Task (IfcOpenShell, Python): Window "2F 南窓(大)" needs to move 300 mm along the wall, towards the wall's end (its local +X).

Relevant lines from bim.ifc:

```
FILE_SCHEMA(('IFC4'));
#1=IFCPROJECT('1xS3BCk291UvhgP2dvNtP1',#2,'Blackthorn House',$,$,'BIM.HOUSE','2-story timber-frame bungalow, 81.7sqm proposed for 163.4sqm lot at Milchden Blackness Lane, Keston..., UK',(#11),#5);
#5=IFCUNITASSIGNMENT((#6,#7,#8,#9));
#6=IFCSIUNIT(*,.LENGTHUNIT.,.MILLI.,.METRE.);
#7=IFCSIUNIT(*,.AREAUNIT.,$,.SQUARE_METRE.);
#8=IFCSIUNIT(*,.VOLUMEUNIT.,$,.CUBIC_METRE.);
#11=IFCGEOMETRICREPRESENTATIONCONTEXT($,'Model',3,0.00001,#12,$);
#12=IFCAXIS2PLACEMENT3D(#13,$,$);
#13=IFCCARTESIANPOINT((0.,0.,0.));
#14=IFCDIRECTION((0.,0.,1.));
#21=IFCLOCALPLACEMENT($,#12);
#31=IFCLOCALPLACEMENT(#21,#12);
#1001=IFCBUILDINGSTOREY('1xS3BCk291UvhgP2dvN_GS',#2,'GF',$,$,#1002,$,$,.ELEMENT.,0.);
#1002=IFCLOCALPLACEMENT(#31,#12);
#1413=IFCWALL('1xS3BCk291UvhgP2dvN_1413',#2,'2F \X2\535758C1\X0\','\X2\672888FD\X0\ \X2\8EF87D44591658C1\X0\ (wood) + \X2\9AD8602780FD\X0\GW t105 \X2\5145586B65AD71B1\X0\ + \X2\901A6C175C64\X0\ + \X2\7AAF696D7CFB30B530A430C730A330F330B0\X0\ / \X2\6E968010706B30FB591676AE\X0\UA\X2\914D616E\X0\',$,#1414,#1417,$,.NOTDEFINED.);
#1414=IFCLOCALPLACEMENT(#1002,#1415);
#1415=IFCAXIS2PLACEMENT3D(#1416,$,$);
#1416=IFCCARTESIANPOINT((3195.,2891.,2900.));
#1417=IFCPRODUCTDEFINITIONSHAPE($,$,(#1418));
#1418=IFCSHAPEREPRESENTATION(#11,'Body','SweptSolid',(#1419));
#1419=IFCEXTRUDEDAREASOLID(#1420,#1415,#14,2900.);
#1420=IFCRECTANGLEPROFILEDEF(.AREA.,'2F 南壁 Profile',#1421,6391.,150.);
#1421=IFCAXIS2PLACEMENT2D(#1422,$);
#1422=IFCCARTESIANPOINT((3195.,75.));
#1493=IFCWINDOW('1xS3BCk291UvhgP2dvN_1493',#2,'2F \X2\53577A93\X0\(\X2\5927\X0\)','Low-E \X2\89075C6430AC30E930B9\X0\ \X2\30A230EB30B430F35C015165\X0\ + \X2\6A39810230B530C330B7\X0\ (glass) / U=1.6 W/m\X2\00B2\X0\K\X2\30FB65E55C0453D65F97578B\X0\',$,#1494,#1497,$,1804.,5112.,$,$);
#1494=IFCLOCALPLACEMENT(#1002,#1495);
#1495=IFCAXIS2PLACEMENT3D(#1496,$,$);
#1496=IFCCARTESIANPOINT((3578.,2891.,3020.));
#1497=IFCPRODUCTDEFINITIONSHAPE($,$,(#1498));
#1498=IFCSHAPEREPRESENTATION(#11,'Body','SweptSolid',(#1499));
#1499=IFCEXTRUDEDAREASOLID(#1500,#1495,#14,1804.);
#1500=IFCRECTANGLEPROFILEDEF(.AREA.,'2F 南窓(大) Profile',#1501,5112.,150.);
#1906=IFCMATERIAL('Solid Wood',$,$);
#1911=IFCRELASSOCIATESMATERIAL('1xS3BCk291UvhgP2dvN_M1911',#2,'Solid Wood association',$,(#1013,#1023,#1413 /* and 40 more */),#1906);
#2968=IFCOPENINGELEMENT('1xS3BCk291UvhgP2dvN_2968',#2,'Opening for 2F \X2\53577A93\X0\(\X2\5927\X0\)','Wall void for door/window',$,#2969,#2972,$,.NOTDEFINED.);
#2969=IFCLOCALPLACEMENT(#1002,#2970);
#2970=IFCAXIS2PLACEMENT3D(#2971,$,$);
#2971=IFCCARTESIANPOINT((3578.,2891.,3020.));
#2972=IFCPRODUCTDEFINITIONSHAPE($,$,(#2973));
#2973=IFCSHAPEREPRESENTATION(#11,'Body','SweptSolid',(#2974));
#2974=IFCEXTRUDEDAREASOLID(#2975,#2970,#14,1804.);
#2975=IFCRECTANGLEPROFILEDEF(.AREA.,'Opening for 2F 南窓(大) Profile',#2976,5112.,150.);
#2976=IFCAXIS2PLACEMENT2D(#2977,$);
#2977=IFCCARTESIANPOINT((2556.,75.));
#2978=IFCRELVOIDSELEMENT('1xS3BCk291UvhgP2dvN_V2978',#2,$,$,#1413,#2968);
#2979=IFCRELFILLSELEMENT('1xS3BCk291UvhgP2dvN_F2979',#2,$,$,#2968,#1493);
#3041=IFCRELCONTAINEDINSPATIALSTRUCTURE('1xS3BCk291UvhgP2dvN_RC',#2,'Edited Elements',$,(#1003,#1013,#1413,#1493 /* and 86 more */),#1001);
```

```python
import ifcopenshell
import ifcopenshell.api.geometry
import ifcopenshell.util.placement
import ifcopenshell.util.unit

model = ifcopenshell.open("bim.ifc")
unit_scale = ifcopenshell.util.unit.calculate_unit_scale(model)

window = model.by_guid("1xS3BCk291UvhgP2dvN_1493")
opening = window.FillsVoids[0].RelatingOpeningElement
wall = opening.VoidsElements[0].RelatingBuildingElement

wall_matrix = ifcopenshell.util.placement.get_local_placement(wall.ObjectPlacement)
shift = wall_matrix[:3, 0] * 0.3 / unit_scale
before = ifcopenshell.util.placement.get_local_placement(window.ObjectPlacement)[:3, 3].copy()

# The window is not placed relative to its opening, so move both.
for product in (opening, window):
    matrix = ifcopenshell.util.placement.get_local_placement(product.ObjectPlacement)
    matrix[:3, 3] += shift
    ifcopenshell.api.geometry.edit_object_placement(model, product=product, matrix=matrix, is_si=False)

after = ifcopenshell.util.placement.get_local_placement(window.ObjectPlacement)[:3, 3]
print("window moved by", (after - before).round(3) + 0.0)

model.write("bim-out.ifc")
```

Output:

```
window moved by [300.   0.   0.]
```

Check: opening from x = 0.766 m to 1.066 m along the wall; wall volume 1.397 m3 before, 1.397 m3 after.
